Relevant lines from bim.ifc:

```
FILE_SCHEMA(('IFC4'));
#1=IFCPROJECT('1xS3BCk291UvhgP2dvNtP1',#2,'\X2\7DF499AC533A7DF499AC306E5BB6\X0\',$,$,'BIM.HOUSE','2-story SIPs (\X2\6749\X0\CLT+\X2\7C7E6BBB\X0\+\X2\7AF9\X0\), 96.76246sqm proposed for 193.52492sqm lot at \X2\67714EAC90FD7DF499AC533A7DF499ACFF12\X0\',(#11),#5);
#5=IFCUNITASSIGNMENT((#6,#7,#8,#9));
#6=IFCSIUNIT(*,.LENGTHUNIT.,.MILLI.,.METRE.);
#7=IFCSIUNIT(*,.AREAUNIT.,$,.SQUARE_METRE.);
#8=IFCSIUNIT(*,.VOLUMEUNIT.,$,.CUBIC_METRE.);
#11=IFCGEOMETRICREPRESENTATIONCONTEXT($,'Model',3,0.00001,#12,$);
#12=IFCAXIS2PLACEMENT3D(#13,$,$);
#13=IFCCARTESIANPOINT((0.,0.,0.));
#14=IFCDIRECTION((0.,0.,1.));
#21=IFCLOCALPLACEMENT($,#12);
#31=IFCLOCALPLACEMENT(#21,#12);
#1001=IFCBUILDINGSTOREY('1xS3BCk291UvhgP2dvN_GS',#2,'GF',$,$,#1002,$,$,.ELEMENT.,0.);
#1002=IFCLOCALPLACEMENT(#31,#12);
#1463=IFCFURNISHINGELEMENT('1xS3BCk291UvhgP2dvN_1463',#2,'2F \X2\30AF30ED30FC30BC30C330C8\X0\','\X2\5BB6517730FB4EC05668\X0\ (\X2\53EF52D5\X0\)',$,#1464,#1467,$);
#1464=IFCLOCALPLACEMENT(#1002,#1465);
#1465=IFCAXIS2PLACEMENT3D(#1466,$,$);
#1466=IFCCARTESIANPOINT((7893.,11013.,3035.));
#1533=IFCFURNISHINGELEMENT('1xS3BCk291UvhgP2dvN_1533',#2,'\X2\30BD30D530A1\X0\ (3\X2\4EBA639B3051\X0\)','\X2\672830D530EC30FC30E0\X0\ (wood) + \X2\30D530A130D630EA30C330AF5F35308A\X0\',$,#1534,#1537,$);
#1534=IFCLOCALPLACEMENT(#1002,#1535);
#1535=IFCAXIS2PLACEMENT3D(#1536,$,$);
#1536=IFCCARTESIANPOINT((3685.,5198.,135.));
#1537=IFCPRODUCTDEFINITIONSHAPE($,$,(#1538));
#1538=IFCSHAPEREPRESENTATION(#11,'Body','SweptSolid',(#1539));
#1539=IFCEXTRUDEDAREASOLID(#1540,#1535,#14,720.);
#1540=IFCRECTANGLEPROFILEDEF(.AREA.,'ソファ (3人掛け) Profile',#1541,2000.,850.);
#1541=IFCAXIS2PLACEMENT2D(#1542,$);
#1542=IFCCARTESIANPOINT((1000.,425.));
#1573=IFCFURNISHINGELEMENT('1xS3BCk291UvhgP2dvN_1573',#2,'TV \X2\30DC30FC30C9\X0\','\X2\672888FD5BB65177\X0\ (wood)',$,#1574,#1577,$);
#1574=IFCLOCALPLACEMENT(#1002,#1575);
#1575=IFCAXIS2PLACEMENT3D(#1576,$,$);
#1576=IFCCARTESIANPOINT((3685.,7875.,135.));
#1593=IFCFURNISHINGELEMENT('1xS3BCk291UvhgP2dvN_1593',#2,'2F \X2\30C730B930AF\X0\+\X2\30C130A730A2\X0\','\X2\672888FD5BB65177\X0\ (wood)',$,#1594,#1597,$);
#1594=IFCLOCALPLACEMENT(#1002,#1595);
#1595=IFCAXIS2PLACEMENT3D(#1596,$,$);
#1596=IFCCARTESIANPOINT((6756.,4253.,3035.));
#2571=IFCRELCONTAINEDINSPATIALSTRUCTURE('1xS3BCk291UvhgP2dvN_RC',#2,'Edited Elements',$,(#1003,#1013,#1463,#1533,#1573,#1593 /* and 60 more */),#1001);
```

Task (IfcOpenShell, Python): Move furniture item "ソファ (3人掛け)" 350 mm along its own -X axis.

```python
import ifcopenshell
import ifcopenshell.api.geometry
import ifcopenshell.util.placement
import ifcopenshell.util.unit

model = ifcopenshell.open("bim.ifc")
unit_scale = ifcopenshell.util.unit.calculate_unit_scale(model)

item = model.by_id(1533)
matrix = ifcopenshell.util.placement.get_local_placement(item.ObjectPlacement)
matrix[:3, 3] -= matrix[:3, 0] * 0.35 / unit_scale
ifcopenshell.api.geometry.edit_object_placement(model, product=item, matrix=matrix, is_si=False)

print(ifcopenshell.util.placement.get_local_placement(item.ObjectPlacement).round(3) + 0.0)

model.write("bim-out.ifc")
```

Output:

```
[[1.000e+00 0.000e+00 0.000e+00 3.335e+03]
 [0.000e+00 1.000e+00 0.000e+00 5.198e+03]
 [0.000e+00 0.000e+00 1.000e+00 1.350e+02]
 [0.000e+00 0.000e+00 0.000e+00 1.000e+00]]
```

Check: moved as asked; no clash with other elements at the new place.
